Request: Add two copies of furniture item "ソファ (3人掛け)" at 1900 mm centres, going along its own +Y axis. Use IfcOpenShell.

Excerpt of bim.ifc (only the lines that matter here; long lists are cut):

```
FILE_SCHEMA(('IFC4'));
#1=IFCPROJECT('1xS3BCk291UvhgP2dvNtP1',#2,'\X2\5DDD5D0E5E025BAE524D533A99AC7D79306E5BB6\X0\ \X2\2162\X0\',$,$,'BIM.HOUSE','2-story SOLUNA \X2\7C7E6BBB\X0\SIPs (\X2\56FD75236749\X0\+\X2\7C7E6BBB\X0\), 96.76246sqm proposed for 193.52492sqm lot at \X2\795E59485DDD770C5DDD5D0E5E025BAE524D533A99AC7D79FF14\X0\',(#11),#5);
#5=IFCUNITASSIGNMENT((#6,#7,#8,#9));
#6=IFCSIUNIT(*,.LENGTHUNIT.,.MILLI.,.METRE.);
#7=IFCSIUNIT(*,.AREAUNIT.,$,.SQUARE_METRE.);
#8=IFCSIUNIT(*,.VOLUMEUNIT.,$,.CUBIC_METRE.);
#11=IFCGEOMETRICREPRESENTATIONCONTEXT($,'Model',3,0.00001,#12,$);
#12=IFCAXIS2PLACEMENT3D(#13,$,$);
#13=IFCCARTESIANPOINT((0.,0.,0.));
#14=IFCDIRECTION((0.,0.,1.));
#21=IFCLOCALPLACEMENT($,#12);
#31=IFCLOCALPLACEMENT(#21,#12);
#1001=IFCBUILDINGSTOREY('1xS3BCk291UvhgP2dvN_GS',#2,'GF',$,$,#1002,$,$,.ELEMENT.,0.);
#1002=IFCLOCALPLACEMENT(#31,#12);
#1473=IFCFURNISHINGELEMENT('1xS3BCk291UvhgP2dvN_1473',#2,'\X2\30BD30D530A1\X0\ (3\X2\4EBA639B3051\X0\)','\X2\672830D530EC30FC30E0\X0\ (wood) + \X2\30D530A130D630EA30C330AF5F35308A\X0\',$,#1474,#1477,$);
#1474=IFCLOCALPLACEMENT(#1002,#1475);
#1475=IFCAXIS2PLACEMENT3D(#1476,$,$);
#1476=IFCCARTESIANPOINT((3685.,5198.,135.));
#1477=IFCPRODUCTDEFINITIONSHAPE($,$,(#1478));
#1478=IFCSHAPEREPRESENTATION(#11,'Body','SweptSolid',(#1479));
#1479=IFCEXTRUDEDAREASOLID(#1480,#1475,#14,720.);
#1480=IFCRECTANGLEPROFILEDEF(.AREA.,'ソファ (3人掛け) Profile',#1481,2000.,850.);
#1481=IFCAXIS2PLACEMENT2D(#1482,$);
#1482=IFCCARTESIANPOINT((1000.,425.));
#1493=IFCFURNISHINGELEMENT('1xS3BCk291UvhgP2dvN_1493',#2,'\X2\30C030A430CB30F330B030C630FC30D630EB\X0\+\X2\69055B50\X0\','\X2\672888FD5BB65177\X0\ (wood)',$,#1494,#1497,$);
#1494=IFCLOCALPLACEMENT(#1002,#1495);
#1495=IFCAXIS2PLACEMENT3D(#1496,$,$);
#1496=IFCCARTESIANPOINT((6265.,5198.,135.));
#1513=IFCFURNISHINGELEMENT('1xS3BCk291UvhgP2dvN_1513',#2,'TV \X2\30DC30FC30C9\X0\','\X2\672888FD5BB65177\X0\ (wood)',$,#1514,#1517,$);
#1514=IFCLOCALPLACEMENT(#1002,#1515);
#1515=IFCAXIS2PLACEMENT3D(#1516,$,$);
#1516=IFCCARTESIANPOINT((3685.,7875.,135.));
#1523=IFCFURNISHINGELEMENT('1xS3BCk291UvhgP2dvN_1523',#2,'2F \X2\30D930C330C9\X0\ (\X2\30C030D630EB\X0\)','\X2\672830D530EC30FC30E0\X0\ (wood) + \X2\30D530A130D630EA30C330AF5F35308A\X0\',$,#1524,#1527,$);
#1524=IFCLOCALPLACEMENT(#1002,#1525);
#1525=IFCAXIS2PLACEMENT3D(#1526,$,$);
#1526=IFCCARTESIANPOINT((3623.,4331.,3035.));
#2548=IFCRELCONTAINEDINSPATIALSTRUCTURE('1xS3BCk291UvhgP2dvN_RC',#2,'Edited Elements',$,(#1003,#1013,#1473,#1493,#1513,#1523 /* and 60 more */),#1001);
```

```python
import ifcopenshell
import ifcopenshell.api.geometry
import ifcopenshell.api.root
import ifcopenshell.util.element
import ifcopenshell.util.placement
import ifcopenshell.util.unit

model = ifcopenshell.open("bim.ifc")
unit_scale = ifcopenshell.util.unit.calculate_unit_scale(model)


def reuse_history(source, copy):
    """copy_class also copies each property set's owner history, people and application; keep the originals."""
    for rel in copy.IsDefinedBy:
        if rel.is_a("IfcRelDefinesByProperties") and (history := rel.RelatingPropertyDefinition.OwnerHistory):
            rel.RelatingPropertyDefinition.OwnerHistory = source.OwnerHistory
            ifcopenshell.util.element.remove_deep2(model, history)


source = model.by_guid("1xS3BCk291UvhgP2dvN_1473")
base = ifcopenshell.util.placement.get_local_placement(source.ObjectPlacement)
step = base[:3, 1] * 1.9 / unit_scale

for i in range(1, 3):
    copy = ifcopenshell.api.root.copy_class(model, product=source)
    copy.Representation = ifcopenshell.util.element.copy_deep(
        model, source.Representation, exclude=["IfcGeometricRepresentationContext", "IfcRepresentationMap"]
    )
    reuse_history(source, copy)
    matrix = base.copy()
    matrix[:3, 3] += i * step
    print("added at", matrix[:3, 3].round(3) + 0.0)
    ifcopenshell.api.geometry.edit_object_placement(model, product=copy, matrix=matrix, is_si=False)

model.write("bim_v2.ifc")
```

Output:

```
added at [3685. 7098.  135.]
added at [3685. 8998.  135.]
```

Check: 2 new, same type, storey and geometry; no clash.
